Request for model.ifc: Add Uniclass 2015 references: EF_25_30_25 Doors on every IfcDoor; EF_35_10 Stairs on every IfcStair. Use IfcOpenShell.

First a look at what the model holds.

```python
import ifcopenshell

model = ifcopenshell.open("model.ifc")
print(model.schema)
print("classifications:", [c.Name for c in model.by_type("IfcClassification")])
for ifc_class in ("IfcDoor", "IfcRoof", "IfcStair", "IfcWall", "IfcWindow"):
    print(ifc_class, len(model.by_type(ifc_class)))
```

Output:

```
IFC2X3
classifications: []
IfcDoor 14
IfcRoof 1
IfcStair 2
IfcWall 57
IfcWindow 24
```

```python
import ifcopenshell
import ifcopenshell.api.classification

model = ifcopenshell.open("model.ifc")

# IFC2X3 requires Source and Edition and has no link from the project to the system.
system = model.create_entity("IfcClassification", Source="NBS", Edition="2015", Name="Uniclass 2015")

codes = {
    "IfcDoor": ("EF_25_30_25", "Doors"),
    "IfcStair": ("EF_35_10", "Stairs"),
}
for ifc_class, (code, name) in codes.items():
    products = model.by_type(ifc_class)
    ifcopenshell.api.classification.add_reference(
        model, products=products, classification=system, identification=code, name=name
    )
    print(code, len(products))

model.write("model_edited.ifc")
```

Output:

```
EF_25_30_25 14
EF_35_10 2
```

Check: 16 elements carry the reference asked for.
